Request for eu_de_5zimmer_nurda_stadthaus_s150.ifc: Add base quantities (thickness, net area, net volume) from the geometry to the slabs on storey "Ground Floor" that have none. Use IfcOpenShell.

First a look at what the model holds.

```python
import ifcopenshell
import ifcopenshell.util.element
import ifcopenshell.util.unit

model = ifcopenshell.open("eu_de_5zimmer_nurda_stadthaus_s150.ifc")
print(model.schema)
for unit_type in ("LENGTHUNIT", "AREAUNIT", "VOLUMEUNIT"):
    print(unit_type, ifcopenshell.util.unit.calculate_unit_scale(model, unit_type))
storey = next(s for s in model.by_type("IfcBuildingStorey") if s.Name == "Ground Floor")
slabs = [e for e in ifcopenshell.util.element.get_decomposition(storey) if e.is_a("IfcSlab")]
for e in sorted(slabs, key=lambda e: e.id()):
    print(e.id(), e.is_a(), e.Name, list(ifcopenshell.util.element.get_psets(e, qtos_only=True)), sep=" | ")
```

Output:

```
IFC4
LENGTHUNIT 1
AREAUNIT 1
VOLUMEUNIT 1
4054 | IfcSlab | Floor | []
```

```python
import ifcopenshell
import ifcopenshell.api.pset
import ifcopenshell.geom
import ifcopenshell.util.element
import ifcopenshell.util.shape
import ifcopenshell.util.unit

model = ifcopenshell.open("eu_de_5zimmer_nurda_stadthaus_s150.ifc")
unit_scale = ifcopenshell.util.unit.calculate_unit_scale(model)
area_scale = ifcopenshell.util.unit.calculate_unit_scale(model, "AREAUNIT")
volume_scale = ifcopenshell.util.unit.calculate_unit_scale(model, "VOLUMEUNIT")
settings = ifcopenshell.geom.settings()

storey = next(s for s in model.by_type("IfcBuildingStorey") if s.Name == "Ground Floor")
slabs = [e for e in ifcopenshell.util.element.get_decomposition(storey) if e.is_a("IfcSlab")]

for e in sorted(slabs, key=lambda e: e.id()):
    if ifcopenshell.util.element.get_psets(e, qtos_only=True, should_inherit=False):
        continue
    # Geometry comes back in metres, in the element's own axes.
    shape = ifcopenshell.geom.create_shape(settings, e)
    values = {
        "Width": ifcopenshell.util.shape.get_z(shape.geometry) / unit_scale,
        "NetArea": ifcopenshell.util.shape.get_footprint_area(shape.geometry) / area_scale,
        "NetVolume": ifcopenshell.util.shape.get_volume(shape.geometry) / volume_scale,
    }
    qto = ifcopenshell.api.pset.add_qto(model, product=e, name="Qto_SlabBaseQuantities")
    ifcopenshell.api.pset.edit_qto(model, qto=qto, properties=values)
    print(e.id(), {k: round(v, 3) for k, v in values.items()})

model.write("eu_de_5zimmer_nurda_stadthaus_s150_updated.ifc")
```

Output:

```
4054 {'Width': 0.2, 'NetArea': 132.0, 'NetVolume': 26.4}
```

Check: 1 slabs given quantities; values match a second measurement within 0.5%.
